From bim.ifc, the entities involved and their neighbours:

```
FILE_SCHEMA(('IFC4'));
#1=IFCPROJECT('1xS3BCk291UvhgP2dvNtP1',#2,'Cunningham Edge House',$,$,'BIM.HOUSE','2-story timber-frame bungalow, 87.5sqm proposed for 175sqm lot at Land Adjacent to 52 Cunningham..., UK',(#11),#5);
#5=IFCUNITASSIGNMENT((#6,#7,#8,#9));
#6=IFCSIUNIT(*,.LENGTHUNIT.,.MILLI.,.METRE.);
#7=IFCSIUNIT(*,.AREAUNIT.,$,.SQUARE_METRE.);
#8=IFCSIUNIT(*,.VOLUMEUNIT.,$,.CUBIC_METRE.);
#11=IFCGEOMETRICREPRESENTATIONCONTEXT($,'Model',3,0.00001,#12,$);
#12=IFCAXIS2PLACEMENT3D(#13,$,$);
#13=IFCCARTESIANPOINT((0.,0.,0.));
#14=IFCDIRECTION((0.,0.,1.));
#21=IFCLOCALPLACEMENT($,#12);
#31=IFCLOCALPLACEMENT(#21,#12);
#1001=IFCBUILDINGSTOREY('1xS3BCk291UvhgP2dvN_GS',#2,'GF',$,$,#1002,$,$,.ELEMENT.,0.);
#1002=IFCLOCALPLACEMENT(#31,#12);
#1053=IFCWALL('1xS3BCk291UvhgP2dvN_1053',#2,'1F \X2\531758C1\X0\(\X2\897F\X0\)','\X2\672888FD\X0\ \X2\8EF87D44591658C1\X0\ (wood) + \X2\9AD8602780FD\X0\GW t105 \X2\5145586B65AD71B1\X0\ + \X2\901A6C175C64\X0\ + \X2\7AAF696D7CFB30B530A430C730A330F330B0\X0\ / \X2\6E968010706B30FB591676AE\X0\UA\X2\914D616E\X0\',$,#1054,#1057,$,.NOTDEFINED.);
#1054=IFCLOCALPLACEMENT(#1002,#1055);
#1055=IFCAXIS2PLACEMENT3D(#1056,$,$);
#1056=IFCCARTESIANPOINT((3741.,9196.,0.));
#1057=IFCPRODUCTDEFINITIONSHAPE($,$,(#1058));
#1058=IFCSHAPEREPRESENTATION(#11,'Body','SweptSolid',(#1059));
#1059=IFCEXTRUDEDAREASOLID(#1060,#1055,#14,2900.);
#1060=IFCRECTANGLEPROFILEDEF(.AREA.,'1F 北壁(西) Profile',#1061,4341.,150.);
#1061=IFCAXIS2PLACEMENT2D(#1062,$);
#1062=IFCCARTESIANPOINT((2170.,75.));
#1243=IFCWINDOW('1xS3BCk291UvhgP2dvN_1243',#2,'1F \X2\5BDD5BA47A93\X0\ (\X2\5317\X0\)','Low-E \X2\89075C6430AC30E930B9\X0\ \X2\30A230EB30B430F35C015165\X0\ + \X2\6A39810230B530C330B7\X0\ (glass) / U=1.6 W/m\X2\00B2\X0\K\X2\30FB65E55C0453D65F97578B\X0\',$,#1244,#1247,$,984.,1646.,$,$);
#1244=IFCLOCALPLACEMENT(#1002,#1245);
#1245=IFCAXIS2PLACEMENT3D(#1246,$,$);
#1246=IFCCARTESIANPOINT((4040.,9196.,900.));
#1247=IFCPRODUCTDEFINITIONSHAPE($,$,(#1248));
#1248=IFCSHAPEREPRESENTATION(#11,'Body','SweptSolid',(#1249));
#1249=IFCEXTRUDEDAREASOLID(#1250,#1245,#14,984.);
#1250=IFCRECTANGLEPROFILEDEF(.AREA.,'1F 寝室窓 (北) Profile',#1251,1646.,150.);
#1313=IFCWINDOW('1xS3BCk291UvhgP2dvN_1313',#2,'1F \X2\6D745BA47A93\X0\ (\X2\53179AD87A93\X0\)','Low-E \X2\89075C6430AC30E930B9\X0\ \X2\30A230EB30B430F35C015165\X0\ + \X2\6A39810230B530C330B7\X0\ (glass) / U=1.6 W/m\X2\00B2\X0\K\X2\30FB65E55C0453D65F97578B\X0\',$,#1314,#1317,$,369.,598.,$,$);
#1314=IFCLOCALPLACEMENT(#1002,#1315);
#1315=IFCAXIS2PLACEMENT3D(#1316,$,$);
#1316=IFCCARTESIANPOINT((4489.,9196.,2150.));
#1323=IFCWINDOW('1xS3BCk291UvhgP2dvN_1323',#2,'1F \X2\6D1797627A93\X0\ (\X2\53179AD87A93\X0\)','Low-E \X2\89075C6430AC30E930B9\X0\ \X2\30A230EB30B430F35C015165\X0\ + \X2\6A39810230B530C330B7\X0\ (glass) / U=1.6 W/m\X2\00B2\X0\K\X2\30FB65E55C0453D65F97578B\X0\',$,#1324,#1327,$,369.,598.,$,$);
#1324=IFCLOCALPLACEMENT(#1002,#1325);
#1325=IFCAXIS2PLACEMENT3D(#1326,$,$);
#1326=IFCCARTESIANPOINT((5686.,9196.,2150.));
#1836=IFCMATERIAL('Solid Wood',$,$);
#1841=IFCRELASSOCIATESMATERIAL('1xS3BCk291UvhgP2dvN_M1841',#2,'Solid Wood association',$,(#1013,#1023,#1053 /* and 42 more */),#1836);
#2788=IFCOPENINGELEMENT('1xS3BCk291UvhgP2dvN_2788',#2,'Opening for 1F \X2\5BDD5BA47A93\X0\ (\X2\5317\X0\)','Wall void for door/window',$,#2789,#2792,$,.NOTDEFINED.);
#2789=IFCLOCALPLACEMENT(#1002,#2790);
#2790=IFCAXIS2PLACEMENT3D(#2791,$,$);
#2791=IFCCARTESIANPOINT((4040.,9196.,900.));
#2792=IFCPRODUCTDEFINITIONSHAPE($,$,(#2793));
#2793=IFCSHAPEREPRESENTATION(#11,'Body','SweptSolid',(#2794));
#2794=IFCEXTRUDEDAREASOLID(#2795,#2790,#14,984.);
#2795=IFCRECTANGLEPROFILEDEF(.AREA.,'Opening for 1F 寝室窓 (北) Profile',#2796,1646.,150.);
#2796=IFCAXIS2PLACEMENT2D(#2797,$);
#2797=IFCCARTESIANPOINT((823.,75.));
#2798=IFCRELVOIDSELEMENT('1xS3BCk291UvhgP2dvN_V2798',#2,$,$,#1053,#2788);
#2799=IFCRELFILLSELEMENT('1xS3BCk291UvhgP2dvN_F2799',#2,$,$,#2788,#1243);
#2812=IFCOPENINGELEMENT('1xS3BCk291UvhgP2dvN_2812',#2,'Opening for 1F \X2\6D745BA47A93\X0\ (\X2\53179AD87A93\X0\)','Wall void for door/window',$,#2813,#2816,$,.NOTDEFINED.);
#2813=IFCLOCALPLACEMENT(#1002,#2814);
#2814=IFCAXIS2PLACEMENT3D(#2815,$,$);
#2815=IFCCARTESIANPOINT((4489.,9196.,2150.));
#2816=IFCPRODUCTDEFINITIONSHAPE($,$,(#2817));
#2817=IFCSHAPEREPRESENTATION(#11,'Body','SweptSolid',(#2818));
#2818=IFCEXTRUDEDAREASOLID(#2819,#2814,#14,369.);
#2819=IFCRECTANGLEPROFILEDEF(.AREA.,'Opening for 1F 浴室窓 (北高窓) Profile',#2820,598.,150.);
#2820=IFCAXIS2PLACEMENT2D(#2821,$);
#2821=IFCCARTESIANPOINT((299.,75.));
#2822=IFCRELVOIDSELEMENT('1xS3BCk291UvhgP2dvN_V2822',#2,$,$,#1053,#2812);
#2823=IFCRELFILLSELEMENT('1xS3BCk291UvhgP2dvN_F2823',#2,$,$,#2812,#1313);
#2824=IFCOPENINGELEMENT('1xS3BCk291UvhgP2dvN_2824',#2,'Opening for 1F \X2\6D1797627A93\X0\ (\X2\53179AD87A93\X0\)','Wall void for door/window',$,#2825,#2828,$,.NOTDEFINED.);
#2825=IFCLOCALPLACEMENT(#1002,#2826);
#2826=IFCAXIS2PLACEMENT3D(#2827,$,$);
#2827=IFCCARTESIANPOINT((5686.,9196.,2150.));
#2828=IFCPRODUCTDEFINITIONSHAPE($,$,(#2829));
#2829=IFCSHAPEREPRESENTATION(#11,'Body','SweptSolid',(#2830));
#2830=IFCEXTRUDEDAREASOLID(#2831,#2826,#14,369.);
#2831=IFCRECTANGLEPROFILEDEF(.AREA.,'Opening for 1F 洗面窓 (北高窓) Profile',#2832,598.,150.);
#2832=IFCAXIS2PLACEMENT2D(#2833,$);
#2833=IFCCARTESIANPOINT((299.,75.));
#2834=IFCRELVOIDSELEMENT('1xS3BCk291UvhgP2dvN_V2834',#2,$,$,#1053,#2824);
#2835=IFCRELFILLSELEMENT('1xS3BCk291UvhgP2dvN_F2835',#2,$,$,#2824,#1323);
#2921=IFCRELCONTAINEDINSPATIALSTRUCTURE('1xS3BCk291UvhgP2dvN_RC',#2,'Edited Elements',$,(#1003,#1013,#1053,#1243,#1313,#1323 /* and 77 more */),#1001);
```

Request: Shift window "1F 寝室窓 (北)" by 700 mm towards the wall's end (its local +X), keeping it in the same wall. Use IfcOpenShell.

```python
import ifcopenshell
import ifcopenshell.api.geometry
import ifcopenshell.util.placement

model = ifcopenshell.open("bim.ifc")

window = model.by_guid("1xS3BCk291UvhgP2dvN_1243")
opening = window.FillsVoids[0].RelatingOpeningElement
wall = opening.VoidsElements[0].RelatingBuildingElement

wall_matrix = ifcopenshell.util.placement.get_local_placement(wall.ObjectPlacement)
shift = wall_matrix[:3, 0] * 700.0
before = ifcopenshell.util.placement.get_local_placement(window.ObjectPlacement)[:3, 3].copy()

# The window is not placed relative to its opening, so move both.
for product in (opening, window):
    matrix = ifcopenshell.util.placement.get_local_placement(product.ObjectPlacement)
    matrix[:3, 3] += shift
    ifcopenshell.api.geometry.edit_object_placement(model, product=product, matrix=matrix, is_si=False)

after = ifcopenshell.util.placement.get_local_placement(window.ObjectPlacement)[:3, 3]
print("window moved by", (after - before).round(3) + 0.0)

model.write("bim_updated.ifc")
```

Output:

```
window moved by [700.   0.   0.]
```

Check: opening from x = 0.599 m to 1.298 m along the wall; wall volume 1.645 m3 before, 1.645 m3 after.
